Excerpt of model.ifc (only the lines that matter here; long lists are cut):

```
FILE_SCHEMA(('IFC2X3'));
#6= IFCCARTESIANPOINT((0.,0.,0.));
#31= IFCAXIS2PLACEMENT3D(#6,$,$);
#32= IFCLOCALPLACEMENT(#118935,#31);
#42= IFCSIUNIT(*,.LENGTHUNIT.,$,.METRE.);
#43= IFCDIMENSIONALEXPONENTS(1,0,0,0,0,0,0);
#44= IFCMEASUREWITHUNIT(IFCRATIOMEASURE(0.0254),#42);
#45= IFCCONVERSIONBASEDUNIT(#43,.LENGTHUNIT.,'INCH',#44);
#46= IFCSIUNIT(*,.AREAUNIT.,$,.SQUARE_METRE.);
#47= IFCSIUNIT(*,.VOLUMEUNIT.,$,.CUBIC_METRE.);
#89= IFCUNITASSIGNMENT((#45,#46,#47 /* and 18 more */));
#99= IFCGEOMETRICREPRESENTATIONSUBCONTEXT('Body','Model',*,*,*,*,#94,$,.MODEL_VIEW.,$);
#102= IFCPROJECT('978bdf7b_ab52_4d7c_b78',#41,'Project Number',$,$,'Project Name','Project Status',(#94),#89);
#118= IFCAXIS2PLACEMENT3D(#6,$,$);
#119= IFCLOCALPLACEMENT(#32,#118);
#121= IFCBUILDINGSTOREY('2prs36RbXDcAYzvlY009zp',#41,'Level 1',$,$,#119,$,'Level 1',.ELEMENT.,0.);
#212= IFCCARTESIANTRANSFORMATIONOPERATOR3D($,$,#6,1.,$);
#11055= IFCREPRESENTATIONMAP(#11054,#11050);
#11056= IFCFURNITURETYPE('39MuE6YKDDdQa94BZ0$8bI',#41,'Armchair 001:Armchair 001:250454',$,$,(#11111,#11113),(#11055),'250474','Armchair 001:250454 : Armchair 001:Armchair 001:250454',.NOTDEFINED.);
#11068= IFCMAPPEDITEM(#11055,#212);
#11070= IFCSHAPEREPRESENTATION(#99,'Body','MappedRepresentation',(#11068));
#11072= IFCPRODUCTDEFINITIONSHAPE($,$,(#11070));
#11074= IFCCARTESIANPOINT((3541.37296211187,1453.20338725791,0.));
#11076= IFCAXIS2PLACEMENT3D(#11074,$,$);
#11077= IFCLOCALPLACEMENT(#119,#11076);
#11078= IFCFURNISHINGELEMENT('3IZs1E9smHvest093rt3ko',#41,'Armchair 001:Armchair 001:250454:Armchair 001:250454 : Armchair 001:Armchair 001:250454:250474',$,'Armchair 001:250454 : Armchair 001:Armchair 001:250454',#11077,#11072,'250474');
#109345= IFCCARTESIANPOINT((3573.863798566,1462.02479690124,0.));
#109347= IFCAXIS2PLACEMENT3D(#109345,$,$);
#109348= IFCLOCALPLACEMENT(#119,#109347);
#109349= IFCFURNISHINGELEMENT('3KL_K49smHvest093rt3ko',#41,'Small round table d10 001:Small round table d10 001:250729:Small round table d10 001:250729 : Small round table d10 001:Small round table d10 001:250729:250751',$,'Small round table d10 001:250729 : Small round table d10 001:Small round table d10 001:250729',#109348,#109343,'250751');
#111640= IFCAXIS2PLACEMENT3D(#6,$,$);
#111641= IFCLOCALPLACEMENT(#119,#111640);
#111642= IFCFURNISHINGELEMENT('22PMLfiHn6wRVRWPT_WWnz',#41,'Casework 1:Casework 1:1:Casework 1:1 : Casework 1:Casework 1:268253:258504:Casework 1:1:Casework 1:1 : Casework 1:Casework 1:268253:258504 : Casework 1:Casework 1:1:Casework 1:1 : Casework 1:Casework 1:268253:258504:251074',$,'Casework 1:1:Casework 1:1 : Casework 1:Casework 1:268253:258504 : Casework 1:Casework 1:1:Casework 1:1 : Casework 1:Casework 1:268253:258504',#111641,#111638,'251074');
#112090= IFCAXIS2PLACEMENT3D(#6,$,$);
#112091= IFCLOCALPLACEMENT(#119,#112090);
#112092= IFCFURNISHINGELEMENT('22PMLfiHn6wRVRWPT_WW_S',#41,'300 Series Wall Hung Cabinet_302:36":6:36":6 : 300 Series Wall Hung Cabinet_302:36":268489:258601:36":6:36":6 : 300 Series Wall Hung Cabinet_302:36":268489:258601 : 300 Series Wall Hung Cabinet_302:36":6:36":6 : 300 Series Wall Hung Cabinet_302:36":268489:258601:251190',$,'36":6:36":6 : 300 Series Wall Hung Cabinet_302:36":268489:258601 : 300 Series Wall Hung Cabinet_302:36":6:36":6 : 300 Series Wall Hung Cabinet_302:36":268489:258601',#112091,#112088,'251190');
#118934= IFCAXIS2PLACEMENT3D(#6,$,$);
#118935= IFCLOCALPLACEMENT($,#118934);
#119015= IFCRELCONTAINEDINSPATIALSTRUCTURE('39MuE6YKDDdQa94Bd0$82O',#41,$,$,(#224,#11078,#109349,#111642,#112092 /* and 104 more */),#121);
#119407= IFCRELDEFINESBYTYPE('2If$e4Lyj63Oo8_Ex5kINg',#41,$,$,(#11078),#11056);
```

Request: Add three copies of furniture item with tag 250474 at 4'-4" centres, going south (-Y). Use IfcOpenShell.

```python
import numpy as np
import ifcopenshell
import ifcopenshell.api.geometry
import ifcopenshell.api.root
import ifcopenshell.util.element
import ifcopenshell.util.placement
import ifcopenshell.util.unit

model = ifcopenshell.open("model.ifc")
unit_scale = ifcopenshell.util.unit.calculate_unit_scale(model)


def reuse_history(source, copy):
    """copy_class also copies each property set's owner history, people and application; keep the originals."""
    for rel in copy.IsDefinedBy:
        if rel.is_a("IfcRelDefinesByProperties") and (history := rel.RelatingPropertyDefinition.OwnerHistory):
            rel.RelatingPropertyDefinition.OwnerHistory = source.OwnerHistory
            ifcopenshell.util.element.remove_deep2(model, history)


source = model.by_guid("3IZs1E9smHvest093rt3ko")
base = ifcopenshell.util.placement.get_local_placement(source.ObjectPlacement)
step = np.array([0.0, -1.0, 0.0]) * 52 * 0.0254 / unit_scale

for i in range(1, 4):
    copy = ifcopenshell.api.root.copy_class(model, product=source)
    copy.Representation = ifcopenshell.util.element.copy_deep(
        model, source.Representation, exclude=["IfcGeometricRepresentationContext", "IfcRepresentationMap"]
    )
    copy.Name = "Armchair 001:Armchair 001:250454:Armchair 001:250454 : Armchair 001:Armchair 001"
    copy.Tag = None
    reuse_history(source, copy)
    matrix = base.copy()
    matrix[:3, 3] += i * step
    print("added at", matrix[:3, 3].round(3) + 0.0)
    ifcopenshell.api.geometry.edit_object_placement(model, product=copy, matrix=matrix, is_si=False)

model.write("model_edited.ifc")
```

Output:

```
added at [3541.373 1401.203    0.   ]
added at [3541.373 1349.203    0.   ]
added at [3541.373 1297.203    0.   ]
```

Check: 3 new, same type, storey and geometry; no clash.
